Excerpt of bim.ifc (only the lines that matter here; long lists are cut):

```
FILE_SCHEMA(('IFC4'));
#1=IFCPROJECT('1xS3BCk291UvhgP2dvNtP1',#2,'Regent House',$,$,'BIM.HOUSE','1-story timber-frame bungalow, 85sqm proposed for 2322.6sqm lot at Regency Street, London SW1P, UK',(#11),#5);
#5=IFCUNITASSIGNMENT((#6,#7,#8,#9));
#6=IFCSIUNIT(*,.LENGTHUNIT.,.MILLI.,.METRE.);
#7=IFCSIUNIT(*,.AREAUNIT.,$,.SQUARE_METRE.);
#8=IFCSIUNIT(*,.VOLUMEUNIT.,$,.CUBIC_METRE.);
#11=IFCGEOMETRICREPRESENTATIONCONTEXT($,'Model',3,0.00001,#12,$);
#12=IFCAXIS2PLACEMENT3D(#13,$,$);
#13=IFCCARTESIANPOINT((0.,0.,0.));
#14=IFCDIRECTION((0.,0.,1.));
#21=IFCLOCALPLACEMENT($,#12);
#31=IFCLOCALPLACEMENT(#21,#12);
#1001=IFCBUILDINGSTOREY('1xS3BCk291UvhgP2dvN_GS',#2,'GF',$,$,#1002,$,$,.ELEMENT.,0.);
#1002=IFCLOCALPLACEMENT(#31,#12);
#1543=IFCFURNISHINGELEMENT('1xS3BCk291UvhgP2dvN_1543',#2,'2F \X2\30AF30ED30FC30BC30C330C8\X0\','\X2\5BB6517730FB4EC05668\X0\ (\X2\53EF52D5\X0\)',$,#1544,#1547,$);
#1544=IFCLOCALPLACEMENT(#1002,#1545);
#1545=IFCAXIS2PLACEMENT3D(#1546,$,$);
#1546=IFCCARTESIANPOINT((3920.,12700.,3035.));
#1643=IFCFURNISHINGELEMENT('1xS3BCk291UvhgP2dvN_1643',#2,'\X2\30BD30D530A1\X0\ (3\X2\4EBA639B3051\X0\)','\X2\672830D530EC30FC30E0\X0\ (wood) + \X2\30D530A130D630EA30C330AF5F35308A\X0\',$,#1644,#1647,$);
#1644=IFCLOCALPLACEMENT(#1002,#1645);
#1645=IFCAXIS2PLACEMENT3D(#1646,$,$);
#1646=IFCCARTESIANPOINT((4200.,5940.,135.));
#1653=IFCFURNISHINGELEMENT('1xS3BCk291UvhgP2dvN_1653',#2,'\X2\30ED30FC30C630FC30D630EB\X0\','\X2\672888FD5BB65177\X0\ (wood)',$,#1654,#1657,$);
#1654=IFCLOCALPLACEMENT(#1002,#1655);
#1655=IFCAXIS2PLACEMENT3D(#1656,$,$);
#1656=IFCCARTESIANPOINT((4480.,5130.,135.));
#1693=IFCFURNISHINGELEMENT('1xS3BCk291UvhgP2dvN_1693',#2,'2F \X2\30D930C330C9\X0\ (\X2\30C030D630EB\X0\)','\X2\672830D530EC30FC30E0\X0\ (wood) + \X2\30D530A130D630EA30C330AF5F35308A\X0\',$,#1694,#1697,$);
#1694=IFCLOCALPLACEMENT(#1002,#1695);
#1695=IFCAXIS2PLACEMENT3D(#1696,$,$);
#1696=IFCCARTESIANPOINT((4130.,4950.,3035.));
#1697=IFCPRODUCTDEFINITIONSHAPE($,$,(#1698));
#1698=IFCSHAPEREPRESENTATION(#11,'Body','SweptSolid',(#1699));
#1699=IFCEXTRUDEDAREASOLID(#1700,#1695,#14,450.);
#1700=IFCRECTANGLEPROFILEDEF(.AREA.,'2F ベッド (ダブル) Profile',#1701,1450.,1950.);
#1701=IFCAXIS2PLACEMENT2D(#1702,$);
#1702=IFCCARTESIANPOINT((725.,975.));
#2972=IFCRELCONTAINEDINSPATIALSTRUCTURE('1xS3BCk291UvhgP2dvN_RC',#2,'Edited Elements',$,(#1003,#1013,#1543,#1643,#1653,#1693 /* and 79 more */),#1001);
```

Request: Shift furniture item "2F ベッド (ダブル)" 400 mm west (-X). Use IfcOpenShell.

```python
import ifcopenshell
import ifcopenshell.api.geometry
import ifcopenshell.util.placement
import ifcopenshell.util.unit

model = ifcopenshell.open("bim.ifc")
unit_scale = ifcopenshell.util.unit.calculate_unit_scale(model)

item = model.by_guid("1xS3BCk291UvhgP2dvN_1693")
matrix = ifcopenshell.util.placement.get_local_placement(item.ObjectPlacement)
matrix[0, 3] -= 0.4 / unit_scale
ifcopenshell.api.geometry.edit_object_placement(model, product=item, matrix=matrix, is_si=False)

print(ifcopenshell.util.placement.get_local_placement(item.ObjectPlacement).round(3) + 0.0)

model.write("bim_rev.ifc")
```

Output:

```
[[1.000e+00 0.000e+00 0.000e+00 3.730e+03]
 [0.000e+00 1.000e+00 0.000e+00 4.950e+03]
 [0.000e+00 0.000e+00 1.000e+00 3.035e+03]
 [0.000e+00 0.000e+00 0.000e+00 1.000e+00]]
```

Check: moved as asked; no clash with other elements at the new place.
